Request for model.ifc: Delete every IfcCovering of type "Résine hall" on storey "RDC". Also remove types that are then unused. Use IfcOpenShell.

First a look at what the model holds.

```python
import ifcopenshell
import ifcopenshell.util.element

model = ifcopenshell.open("model.ifc")
print(model.schema)
storey = next(s for s in model.by_type("IfcBuildingStorey") if s.Name == "RDC")
coverings = [e for e in ifcopenshell.util.element.get_decomposition(storey) if e.is_a("IfcCovering")]
seen = {}
for e in coverings:
    element_type = ifcopenshell.util.element.get_type(e)
    name = element_type.Name if element_type not in (None, e) else None
    seen[name] = seen.get(name, 0) + 1
for name, count in sorted(seen.items(), key=str):
    print(count, "x", name)
```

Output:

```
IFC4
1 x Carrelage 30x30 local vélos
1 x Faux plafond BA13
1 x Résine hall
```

```python
import ifcopenshell
import ifcopenshell.api.root
import ifcopenshell.util.element

model = ifcopenshell.open("model.ifc")

storey = next(s for s in model.by_type("IfcBuildingStorey") if s.Name == "RDC")
coverings = [e for e in ifcopenshell.util.element.get_decomposition(storey) if e.is_a("IfcCovering")]
targets = [e for e in coverings if (t := ifcopenshell.util.element.get_type(e)) not in (None, e) and t.Name == "Résine hall"]
types = {ifcopenshell.util.element.get_type(e) for e in targets} - {None, *targets}

for e in targets:
    ifcopenshell.api.root.remove_product(model, product=e)
print(len(targets), "removed")

unused = [t for t in types if not ifcopenshell.util.element.get_types(t)]
for t in unused:
    ifcopenshell.api.root.remove_product(model, product=t)
print(len(unused), "unused types removed")

model.write("model_v2.ifc")
```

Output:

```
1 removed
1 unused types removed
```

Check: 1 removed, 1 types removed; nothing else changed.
